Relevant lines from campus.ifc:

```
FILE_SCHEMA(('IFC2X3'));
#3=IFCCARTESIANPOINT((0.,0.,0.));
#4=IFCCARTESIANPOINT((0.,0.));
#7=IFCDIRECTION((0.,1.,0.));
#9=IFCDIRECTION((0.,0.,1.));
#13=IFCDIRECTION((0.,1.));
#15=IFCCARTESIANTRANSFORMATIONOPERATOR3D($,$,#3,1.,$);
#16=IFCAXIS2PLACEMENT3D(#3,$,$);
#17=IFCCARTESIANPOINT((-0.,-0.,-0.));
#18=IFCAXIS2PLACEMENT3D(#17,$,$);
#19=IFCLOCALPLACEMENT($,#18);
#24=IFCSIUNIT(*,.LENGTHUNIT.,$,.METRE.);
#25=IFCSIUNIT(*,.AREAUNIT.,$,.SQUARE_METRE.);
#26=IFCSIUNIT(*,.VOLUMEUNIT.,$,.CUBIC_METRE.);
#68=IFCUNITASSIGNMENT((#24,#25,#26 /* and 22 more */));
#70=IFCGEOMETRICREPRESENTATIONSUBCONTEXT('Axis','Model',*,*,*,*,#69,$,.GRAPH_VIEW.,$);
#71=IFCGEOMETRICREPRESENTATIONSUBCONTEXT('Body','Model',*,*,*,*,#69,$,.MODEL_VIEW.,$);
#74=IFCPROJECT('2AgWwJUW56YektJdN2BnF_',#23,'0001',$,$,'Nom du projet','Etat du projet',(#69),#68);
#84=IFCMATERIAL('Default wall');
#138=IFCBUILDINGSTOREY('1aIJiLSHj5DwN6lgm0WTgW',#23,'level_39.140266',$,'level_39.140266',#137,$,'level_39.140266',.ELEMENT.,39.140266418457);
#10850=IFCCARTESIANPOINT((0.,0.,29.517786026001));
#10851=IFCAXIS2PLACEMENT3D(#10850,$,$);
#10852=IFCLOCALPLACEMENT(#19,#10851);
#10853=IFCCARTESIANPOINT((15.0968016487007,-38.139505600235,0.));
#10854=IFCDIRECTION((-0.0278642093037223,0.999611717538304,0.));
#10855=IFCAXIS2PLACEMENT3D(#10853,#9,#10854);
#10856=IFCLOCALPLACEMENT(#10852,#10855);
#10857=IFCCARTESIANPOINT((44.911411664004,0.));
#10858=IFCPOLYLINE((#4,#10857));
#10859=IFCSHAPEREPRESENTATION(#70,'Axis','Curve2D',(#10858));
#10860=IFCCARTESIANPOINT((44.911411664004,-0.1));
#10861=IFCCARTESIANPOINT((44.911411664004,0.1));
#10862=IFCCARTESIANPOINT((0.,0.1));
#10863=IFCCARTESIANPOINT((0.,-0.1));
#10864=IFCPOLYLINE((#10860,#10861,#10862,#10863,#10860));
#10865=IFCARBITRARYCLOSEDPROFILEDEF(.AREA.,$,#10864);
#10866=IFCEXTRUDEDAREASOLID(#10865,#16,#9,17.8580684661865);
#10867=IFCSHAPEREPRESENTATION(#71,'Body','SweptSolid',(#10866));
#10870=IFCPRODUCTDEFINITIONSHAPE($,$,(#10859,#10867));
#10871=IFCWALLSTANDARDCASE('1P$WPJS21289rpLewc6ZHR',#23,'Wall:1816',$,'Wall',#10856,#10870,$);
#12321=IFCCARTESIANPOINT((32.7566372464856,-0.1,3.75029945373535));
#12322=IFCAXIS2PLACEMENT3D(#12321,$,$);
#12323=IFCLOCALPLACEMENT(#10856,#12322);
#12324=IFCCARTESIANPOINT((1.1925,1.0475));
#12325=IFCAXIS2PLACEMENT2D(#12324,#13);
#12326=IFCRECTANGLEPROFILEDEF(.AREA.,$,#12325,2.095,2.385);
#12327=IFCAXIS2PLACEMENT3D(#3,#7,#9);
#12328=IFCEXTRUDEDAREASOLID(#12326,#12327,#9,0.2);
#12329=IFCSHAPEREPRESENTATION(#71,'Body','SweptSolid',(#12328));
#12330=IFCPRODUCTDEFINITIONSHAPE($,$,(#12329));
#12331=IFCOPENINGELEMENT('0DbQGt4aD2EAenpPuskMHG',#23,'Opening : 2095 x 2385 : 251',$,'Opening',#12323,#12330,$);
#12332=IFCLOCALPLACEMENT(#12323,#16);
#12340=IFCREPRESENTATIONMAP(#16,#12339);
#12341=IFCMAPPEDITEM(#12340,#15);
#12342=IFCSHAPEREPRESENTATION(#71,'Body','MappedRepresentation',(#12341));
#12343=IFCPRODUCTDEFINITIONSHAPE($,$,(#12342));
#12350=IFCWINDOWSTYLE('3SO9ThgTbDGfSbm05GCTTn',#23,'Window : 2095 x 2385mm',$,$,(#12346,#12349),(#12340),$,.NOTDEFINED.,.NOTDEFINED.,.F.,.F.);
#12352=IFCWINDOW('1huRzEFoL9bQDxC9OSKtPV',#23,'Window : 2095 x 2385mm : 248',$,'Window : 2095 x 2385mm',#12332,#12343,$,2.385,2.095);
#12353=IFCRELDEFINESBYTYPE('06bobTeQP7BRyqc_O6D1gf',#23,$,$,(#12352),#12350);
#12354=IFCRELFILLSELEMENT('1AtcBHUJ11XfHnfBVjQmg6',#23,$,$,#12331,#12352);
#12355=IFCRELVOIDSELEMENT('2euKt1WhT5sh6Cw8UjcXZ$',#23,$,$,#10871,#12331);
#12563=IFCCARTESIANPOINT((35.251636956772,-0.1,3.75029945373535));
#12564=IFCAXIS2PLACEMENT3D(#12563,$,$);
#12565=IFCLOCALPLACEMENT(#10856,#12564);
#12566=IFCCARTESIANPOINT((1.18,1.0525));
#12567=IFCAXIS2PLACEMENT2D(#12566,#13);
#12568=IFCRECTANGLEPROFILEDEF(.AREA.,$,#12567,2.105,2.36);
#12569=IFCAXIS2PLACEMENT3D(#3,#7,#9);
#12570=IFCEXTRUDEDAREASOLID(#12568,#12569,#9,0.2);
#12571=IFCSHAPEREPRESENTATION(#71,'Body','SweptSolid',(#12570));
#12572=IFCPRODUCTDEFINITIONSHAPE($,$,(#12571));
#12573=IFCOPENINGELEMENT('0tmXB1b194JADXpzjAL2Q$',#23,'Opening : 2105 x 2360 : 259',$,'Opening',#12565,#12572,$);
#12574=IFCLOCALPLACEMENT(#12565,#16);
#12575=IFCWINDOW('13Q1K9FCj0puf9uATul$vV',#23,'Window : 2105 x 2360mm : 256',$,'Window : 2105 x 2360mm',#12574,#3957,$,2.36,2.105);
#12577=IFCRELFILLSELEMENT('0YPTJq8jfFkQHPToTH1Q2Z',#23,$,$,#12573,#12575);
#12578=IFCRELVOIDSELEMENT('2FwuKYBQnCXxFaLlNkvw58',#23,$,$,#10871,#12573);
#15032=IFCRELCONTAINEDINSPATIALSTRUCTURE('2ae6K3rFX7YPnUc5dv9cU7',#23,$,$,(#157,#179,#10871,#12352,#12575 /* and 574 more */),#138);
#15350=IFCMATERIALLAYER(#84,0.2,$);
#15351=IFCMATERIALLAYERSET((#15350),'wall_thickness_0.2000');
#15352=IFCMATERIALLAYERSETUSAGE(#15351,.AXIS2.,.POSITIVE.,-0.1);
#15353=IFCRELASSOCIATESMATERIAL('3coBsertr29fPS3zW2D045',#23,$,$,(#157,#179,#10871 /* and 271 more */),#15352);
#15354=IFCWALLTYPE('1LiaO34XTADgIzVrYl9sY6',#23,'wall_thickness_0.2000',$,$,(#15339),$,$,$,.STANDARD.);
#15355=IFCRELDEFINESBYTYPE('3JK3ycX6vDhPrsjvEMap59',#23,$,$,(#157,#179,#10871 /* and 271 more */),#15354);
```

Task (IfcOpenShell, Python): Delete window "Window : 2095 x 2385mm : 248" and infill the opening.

```python
import ifcopenshell
import ifcopenshell.api.feature
import ifcopenshell.api.root
import ifcopenshell.geom
import ifcopenshell.util.shape

model = ifcopenshell.open("campus.ifc")
settings = ifcopenshell.geom.settings()


def volume(element):
    """Net volume in cubic metres, openings subtracted."""
    shape = ifcopenshell.geom.create_shape(settings, element)
    return ifcopenshell.util.shape.get_volume(shape.geometry)


window = model.by_guid("1huRzEFoL9bQDxC9OSKtPV")
opening = window.FillsVoids[0].RelatingOpeningElement
wall = opening.VoidsElements[0].RelatingBuildingElement
before = volume(wall)

ifcopenshell.api.root.remove_product(model, product=window)
ifcopenshell.api.feature.remove_feature(model, feature=opening)

after = volume(wall)

print(f"wall volume {before:.3f} -> {after:.3f} m3")

model.write("campus-out.ifc")
```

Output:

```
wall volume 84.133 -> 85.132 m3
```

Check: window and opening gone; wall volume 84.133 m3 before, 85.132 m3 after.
